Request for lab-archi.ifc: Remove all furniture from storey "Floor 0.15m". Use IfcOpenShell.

First a look at what the model holds.

```python
import ifcopenshell
import ifcopenshell.util.element

model = ifcopenshell.open("lab-archi.ifc")
print(model.schema)
storey = next(s for s in model.by_type("IfcBuildingStorey") if s.Name == "Floor 0.15m")
furniture = [e for e in ifcopenshell.util.element.get_decomposition(storey) if e.is_a("IfcFurnishingElement")]
seen = {}
for e in furniture:
    element_type = ifcopenshell.util.element.get_type(e)
    name = element_type.Name if element_type not in (None, e) else None
    seen[name] = seen.get(name, 0) + 1
for name, count in sorted(seen.items(), key=str):
    print(count, "x", name)
```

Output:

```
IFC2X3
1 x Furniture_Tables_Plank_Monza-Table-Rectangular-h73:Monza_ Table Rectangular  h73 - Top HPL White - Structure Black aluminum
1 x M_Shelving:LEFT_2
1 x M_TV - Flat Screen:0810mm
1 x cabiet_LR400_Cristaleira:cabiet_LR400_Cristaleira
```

```python
import ifcopenshell
import ifcopenshell.api.root
import ifcopenshell.util.element

model = ifcopenshell.open("lab-archi.ifc")

storey = next(s for s in model.by_type("IfcBuildingStorey") if s.Name == "Floor 0.15m")
furniture = [e for e in ifcopenshell.util.element.get_decomposition(storey) if e.is_a("IfcFurnishingElement")]

for e in furniture:
    ifcopenshell.api.root.remove_product(model, product=e)
print(len(furniture), "removed")

model.write("lab-archi-out.ifc")
```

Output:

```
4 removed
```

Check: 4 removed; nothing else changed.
